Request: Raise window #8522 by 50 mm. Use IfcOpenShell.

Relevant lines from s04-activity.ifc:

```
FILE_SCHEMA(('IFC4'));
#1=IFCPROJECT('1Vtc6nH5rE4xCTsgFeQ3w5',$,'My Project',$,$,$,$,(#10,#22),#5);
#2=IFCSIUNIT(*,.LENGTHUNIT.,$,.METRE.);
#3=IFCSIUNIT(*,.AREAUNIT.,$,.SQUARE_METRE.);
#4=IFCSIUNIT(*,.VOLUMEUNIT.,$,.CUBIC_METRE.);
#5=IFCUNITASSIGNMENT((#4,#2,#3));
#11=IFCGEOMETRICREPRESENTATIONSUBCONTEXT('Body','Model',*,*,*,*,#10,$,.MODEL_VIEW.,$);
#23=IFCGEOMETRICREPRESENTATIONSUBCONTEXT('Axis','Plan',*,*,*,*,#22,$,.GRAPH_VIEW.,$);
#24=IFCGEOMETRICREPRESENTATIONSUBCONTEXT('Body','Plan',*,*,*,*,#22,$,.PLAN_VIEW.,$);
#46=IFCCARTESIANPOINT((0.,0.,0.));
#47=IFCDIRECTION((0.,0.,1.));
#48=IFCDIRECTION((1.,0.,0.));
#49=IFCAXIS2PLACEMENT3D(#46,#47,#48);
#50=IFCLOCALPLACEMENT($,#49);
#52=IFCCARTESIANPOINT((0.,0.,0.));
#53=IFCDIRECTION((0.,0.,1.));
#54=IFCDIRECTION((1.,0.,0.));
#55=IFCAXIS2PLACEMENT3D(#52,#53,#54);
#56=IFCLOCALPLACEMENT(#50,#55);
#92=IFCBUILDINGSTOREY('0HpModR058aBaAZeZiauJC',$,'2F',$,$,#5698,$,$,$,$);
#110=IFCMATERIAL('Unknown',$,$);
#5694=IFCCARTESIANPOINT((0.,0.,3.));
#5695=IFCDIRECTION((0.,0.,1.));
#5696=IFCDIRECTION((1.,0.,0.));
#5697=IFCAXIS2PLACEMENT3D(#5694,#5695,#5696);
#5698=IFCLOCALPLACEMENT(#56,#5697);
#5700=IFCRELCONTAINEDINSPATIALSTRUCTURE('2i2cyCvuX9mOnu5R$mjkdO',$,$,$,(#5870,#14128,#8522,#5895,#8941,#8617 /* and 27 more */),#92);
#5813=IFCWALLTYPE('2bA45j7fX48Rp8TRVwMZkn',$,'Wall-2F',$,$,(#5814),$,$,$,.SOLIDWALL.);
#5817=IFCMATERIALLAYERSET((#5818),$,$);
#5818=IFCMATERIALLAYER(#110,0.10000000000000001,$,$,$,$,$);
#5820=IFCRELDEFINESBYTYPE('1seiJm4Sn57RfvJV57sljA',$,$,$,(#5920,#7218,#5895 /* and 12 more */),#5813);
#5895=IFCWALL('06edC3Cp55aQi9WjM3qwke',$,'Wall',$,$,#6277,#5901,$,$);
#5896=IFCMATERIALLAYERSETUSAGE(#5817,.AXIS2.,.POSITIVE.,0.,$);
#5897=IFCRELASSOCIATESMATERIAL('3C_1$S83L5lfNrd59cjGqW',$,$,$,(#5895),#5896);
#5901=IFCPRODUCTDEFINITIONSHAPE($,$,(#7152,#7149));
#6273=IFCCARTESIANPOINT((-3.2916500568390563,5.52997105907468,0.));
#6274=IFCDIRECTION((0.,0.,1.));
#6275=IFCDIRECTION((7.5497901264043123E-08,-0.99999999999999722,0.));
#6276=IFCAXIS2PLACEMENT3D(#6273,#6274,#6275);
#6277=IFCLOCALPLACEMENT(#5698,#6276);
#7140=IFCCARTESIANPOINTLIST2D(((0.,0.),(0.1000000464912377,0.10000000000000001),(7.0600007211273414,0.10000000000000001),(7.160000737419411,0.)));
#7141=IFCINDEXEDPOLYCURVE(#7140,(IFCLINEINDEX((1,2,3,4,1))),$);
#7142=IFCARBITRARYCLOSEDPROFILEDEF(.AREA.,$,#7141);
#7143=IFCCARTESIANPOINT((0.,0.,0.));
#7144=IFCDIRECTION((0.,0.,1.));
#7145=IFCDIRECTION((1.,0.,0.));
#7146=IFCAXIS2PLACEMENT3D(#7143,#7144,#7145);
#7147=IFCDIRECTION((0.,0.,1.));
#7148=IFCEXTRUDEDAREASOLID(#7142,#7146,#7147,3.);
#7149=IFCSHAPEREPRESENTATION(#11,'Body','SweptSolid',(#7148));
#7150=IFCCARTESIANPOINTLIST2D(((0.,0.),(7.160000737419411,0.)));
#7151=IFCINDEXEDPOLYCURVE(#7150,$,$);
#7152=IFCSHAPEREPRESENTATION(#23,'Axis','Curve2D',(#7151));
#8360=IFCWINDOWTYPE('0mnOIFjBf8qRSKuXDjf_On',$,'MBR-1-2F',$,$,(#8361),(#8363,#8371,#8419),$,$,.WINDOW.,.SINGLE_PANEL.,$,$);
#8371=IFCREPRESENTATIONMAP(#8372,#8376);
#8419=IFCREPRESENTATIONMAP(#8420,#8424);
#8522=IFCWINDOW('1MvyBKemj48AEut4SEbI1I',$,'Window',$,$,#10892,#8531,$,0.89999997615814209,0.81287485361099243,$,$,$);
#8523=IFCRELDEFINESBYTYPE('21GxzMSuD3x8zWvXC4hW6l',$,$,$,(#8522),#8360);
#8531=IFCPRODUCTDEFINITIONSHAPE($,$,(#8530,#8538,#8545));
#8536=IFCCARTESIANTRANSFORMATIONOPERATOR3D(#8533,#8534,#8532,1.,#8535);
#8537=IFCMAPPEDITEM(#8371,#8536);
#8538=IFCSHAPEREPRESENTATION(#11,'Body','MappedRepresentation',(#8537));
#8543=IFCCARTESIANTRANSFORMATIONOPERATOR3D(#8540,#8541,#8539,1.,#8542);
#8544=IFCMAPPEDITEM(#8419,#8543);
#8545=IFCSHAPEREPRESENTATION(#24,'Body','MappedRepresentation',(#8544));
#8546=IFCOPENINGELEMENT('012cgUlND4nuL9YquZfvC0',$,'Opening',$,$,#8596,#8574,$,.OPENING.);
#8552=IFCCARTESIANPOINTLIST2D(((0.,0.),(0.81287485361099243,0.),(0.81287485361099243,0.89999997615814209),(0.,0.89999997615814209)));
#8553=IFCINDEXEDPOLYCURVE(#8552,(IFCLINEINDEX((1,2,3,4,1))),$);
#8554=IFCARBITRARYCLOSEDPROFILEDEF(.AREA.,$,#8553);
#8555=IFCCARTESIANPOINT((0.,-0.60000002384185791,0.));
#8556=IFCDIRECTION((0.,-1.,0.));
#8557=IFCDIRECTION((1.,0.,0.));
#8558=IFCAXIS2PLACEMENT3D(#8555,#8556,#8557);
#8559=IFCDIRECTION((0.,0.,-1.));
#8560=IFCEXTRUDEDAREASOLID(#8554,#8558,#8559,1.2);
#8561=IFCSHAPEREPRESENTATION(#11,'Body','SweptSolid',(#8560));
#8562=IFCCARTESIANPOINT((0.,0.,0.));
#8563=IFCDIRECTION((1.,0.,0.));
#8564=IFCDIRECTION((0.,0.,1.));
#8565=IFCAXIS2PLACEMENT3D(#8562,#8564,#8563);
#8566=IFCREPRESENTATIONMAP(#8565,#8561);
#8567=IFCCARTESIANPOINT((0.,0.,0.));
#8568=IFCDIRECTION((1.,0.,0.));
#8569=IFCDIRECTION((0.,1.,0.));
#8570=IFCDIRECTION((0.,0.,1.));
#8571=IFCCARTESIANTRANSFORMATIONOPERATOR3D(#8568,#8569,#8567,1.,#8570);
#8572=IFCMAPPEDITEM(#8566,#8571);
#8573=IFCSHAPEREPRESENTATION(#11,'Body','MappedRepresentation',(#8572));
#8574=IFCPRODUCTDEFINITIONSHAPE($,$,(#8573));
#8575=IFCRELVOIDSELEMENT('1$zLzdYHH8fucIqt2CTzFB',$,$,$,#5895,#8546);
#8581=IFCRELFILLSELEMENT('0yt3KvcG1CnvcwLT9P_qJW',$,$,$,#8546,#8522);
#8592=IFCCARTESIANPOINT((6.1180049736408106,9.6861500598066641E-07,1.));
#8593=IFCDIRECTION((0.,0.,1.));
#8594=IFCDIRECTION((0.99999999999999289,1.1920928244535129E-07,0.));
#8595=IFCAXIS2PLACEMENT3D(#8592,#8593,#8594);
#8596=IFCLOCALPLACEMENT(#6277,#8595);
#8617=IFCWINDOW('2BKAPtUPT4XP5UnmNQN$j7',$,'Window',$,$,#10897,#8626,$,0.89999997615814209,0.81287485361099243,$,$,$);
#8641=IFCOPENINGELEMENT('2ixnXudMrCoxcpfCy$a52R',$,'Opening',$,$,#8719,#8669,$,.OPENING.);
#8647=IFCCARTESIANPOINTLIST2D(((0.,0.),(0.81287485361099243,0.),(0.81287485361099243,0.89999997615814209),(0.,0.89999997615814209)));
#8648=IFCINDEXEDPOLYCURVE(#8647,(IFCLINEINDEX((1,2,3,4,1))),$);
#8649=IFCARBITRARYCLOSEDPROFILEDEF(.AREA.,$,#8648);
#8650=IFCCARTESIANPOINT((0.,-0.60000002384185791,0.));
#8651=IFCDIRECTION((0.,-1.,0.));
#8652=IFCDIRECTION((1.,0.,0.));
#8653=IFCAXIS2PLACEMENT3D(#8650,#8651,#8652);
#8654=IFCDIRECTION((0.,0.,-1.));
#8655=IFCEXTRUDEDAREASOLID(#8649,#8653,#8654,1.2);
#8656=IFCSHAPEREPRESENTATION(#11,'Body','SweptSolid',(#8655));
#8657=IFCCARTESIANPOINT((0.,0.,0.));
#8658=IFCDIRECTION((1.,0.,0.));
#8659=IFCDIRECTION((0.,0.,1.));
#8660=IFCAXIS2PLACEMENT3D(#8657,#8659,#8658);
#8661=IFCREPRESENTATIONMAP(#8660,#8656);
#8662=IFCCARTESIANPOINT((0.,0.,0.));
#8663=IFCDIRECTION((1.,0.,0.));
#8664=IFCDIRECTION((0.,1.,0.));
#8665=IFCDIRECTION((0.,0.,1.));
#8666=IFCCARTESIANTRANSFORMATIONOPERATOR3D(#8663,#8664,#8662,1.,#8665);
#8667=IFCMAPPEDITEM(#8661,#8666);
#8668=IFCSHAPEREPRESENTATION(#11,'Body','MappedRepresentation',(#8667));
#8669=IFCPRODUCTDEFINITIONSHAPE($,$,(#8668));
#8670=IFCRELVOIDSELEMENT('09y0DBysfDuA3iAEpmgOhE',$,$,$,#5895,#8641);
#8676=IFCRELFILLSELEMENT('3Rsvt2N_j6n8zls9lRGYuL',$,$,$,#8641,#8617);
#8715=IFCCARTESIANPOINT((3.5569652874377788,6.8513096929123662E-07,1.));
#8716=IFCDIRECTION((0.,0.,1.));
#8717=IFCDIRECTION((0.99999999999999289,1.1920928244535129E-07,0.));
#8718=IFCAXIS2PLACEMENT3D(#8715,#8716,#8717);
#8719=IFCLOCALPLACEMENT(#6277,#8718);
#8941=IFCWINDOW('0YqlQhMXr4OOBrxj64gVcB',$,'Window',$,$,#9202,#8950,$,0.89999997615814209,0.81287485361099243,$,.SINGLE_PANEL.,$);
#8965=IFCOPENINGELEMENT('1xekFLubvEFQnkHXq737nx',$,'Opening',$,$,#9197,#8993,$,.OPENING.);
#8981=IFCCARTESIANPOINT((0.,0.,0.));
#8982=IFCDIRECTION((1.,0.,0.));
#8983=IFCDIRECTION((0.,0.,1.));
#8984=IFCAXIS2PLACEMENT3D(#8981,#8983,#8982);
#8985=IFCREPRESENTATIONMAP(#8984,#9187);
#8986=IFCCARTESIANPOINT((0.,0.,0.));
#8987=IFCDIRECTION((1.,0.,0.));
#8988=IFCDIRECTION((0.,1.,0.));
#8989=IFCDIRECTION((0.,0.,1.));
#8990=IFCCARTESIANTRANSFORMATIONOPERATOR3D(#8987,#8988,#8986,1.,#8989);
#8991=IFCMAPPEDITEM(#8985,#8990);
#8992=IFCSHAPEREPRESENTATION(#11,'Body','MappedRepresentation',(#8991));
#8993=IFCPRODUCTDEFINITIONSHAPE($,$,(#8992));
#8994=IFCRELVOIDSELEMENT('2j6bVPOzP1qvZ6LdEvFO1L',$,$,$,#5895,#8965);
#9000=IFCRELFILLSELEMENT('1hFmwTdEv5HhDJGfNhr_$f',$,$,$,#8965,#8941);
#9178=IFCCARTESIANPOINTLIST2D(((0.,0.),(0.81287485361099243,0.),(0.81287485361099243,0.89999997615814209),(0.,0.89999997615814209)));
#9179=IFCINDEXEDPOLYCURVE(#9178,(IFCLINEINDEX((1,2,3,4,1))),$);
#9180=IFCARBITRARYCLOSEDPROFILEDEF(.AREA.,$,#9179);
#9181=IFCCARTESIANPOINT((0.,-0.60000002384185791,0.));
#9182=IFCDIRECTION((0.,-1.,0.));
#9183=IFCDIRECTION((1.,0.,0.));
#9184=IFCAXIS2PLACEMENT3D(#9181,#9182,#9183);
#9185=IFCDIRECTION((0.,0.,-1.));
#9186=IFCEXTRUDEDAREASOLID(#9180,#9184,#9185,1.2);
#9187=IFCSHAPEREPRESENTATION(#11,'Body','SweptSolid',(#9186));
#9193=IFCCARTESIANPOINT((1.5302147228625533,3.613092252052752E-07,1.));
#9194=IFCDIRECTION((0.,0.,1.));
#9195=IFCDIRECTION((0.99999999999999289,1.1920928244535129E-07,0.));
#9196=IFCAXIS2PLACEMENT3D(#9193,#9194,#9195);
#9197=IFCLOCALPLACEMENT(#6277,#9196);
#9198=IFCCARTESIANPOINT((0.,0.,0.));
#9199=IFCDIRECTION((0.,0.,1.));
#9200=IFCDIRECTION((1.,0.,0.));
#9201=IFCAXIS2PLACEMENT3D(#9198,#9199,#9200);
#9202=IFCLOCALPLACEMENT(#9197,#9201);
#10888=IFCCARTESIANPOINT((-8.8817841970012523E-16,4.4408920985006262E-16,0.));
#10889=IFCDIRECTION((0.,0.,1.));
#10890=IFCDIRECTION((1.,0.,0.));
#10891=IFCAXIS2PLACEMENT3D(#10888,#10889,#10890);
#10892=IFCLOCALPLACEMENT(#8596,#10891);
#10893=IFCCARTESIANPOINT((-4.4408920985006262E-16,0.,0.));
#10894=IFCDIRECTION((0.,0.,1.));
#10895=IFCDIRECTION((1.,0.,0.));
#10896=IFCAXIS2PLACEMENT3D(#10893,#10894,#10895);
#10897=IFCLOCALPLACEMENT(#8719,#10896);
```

```python
import numpy as np
import ifcopenshell
import ifcopenshell.api.geometry
import ifcopenshell.util.placement
import ifcopenshell.util.unit

model = ifcopenshell.open("s04-activity.ifc")
unit_scale = ifcopenshell.util.unit.calculate_unit_scale(model)

window = model.by_id(8522)
opening = window.FillsVoids[0].RelatingOpeningElement
dz = 0.05 / unit_scale

shift = np.array([0.0, 0.0, dz])
# The window is placed relative to its opening, so it follows when the opening moves.
matrix = ifcopenshell.util.placement.get_local_placement(opening.ObjectPlacement)
matrix[:3, 3] += shift
ifcopenshell.api.geometry.edit_object_placement(
    model, product=opening, matrix=matrix, is_si=False, should_transform_children=True
)

print(f"moved by {dz * unit_scale:+.3f} m")

model.write("s04-activity_updated.ifc")
```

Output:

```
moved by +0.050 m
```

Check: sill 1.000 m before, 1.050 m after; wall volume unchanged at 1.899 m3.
